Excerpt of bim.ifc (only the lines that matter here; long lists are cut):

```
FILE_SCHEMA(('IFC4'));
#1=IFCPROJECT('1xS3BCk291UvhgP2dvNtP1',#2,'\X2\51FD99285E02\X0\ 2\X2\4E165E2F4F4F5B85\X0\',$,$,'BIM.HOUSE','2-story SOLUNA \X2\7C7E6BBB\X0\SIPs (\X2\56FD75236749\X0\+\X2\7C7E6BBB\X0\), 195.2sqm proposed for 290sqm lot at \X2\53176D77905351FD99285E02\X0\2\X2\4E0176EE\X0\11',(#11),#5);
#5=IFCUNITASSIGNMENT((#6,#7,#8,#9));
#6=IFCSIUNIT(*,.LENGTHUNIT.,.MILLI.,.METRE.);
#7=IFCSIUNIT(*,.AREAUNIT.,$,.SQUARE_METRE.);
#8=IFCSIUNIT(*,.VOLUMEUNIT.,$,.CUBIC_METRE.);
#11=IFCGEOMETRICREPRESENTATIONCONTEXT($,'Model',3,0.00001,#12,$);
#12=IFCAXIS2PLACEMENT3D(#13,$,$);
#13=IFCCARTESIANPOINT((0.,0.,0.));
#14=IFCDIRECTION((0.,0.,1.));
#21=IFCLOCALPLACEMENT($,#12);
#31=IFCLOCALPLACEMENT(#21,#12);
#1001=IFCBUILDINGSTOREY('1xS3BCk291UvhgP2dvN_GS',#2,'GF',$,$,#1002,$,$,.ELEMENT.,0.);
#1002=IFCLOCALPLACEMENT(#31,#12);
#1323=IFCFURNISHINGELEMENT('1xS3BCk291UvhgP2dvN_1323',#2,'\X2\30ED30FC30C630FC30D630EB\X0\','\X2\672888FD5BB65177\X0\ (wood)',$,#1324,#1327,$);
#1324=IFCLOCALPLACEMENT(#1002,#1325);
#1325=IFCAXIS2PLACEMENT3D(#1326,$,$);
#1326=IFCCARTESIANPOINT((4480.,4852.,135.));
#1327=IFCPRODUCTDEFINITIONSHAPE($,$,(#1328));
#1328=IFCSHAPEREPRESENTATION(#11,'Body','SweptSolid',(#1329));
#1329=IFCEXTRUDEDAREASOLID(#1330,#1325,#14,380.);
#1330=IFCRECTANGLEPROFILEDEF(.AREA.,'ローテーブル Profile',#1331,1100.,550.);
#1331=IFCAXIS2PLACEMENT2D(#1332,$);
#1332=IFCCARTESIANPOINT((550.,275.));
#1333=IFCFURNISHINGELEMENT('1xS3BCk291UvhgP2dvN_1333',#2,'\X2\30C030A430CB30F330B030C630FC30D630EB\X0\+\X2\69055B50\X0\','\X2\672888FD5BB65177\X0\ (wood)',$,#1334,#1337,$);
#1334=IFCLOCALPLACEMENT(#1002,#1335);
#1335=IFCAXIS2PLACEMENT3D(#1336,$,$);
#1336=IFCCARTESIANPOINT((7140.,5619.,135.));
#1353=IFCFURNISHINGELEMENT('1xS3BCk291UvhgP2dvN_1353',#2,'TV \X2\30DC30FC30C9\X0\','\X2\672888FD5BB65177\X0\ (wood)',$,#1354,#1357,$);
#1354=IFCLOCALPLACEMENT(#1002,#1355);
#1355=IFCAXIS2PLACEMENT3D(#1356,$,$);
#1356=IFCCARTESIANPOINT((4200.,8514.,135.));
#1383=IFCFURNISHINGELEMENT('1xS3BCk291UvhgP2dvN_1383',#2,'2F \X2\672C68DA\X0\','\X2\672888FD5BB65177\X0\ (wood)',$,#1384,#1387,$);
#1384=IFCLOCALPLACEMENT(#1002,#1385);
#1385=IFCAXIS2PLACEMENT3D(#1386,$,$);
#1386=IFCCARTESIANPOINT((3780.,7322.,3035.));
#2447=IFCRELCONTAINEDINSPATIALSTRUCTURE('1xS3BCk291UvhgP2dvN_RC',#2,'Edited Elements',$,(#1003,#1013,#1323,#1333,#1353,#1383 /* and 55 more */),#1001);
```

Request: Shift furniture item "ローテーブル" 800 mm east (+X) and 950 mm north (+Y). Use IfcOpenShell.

```python
import ifcopenshell
import ifcopenshell.api.geometry
import ifcopenshell.util.placement

model = ifcopenshell.open("bim.ifc")

item = model.by_guid("1xS3BCk291UvhgP2dvN_1323")
matrix = ifcopenshell.util.placement.get_local_placement(item.ObjectPlacement)
matrix[0, 3] += 800.0
matrix[1, 3] += 950.0
ifcopenshell.api.geometry.edit_object_placement(model, product=item, matrix=matrix, is_si=False)

print(ifcopenshell.util.placement.get_local_placement(item.ObjectPlacement).round(3) + 0.0)

model.write("bim-out.ifc")
```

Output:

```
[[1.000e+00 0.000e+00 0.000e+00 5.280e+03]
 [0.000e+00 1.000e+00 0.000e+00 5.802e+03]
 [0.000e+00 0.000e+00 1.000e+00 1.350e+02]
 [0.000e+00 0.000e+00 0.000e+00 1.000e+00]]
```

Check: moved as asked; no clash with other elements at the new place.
